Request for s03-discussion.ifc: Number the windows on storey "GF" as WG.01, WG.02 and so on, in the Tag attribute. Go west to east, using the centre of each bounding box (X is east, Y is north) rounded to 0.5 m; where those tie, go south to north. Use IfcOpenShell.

First a look at what the model holds.

```python
import ifcopenshell
import ifcopenshell.util.element
import ifcopenshell.util.placement

model = ifcopenshell.open("s03-discussion.ifc")
print(model.schema)
storey = next(s for s in model.by_type("IfcBuildingStorey") if s.Name == "GF")
windows = [e for e in ifcopenshell.util.element.get_decomposition(storey) if e.is_a("IfcWindow")]
for e in sorted(windows, key=lambda e: e.id()):
    origin = ifcopenshell.util.placement.get_local_placement(e.ObjectPlacement)[:3, 3]
    print(e.id(), e.Tag, e.Name, origin.round(2) + 0.0, sep=" | ")
```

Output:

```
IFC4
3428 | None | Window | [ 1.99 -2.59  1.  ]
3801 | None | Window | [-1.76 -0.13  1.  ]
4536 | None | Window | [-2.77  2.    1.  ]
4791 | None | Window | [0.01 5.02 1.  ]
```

```python
import ifcopenshell
import ifcopenshell.geom
import ifcopenshell.util.element
import ifcopenshell.util.shape

model = ifcopenshell.open("s03-discussion.ifc")
settings = ifcopenshell.geom.settings()
settings.set("use-world-coords", True)


def centre(element):
    shape = ifcopenshell.geom.create_shape(settings, element)
    return ifcopenshell.util.shape.get_bbox_centroid(shape.geometry)


storey = next(s for s in model.by_type("IfcBuildingStorey") if s.Name == "GF")
windows = [e for e in ifcopenshell.util.element.get_decomposition(storey) if e.is_a("IfcWindow")]

# Insertion points can sit at a corner or the storey origin, so sort by the geometry (in metres).
centres = {e: centre(e) for e in windows}
windows.sort(key=lambda e: (round(centres[e][0] / 0.5), centres[e][1]))

for i, e in enumerate(windows, start=1):
    number = f"WG.{i:02d}"
    e.Tag = number
    print(e.id(), number)

model.write("s03-discussion_updated.ifc")
```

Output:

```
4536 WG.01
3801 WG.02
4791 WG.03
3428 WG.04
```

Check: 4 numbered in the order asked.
